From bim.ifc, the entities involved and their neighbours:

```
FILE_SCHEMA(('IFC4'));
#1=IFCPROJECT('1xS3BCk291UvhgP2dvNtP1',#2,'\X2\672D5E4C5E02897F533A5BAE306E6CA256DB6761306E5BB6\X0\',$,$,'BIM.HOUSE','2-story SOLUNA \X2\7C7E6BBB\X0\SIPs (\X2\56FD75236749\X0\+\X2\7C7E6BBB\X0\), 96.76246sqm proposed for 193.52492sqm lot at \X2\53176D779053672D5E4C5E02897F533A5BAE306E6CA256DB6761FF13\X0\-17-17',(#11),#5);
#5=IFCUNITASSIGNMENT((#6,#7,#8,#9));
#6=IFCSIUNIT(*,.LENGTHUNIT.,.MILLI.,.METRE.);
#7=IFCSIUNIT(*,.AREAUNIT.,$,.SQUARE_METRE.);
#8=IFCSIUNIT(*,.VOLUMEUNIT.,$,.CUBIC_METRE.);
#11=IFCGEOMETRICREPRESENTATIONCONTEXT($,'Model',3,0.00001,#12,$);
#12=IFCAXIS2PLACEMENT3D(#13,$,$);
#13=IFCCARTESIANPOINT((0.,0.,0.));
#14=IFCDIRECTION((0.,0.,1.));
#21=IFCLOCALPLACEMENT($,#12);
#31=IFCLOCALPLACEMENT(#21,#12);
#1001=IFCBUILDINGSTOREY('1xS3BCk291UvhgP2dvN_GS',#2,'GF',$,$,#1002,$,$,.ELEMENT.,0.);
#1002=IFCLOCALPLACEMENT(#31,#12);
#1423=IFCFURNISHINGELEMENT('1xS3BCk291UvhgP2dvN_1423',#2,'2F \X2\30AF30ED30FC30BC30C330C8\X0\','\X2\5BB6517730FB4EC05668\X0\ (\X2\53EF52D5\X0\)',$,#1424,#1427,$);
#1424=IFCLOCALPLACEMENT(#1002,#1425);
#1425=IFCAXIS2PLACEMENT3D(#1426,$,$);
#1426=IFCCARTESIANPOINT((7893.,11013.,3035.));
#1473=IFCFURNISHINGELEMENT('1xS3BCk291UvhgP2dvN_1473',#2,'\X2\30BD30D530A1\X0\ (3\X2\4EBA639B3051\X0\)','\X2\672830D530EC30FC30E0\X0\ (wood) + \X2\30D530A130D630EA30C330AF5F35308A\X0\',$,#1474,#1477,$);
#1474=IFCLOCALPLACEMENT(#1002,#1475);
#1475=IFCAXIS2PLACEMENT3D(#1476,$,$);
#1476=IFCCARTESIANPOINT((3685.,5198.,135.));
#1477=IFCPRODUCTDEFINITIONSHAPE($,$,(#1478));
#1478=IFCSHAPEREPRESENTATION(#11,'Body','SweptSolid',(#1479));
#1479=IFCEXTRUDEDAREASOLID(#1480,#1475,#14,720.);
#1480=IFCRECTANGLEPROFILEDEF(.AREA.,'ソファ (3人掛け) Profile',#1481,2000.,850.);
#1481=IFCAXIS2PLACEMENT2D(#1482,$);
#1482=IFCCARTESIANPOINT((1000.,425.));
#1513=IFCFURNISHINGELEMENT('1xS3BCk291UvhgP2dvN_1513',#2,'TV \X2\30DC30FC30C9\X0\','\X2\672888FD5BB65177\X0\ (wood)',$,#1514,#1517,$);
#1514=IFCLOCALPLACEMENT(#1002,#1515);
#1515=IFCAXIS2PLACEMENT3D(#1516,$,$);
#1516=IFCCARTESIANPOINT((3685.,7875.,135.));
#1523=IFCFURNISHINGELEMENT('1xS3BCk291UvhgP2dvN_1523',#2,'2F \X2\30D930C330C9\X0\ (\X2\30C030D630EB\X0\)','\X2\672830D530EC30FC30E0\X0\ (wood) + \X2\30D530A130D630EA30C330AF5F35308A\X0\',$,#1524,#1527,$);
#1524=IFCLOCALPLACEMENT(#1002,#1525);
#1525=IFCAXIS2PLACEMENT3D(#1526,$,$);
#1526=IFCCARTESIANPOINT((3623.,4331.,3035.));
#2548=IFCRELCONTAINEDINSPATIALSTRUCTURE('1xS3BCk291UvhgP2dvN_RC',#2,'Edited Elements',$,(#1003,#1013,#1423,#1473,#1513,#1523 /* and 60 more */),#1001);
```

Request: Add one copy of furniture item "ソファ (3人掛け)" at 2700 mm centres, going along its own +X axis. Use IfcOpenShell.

```python
import ifcopenshell
import ifcopenshell.api.geometry
import ifcopenshell.api.root
import ifcopenshell.util.element
import ifcopenshell.util.placement
import ifcopenshell.util.unit

model = ifcopenshell.open("bim.ifc")
unit_scale = ifcopenshell.util.unit.calculate_unit_scale(model)


def reuse_history(source, copy):
    """copy_class also copies each property set's owner history, people and application; keep the originals."""
    for rel in copy.IsDefinedBy:
        if rel.is_a("IfcRelDefinesByProperties") and (history := rel.RelatingPropertyDefinition.OwnerHistory):
            rel.RelatingPropertyDefinition.OwnerHistory = source.OwnerHistory
            ifcopenshell.util.element.remove_deep2(model, history)


source = model.by_guid("1xS3BCk291UvhgP2dvN_1473")
base = ifcopenshell.util.placement.get_local_placement(source.ObjectPlacement)
step = base[:3, 0] * 2.7 / unit_scale

for i in range(1, 2):
    copy = ifcopenshell.api.root.copy_class(model, product=source)
    copy.Representation = ifcopenshell.util.element.copy_deep(
        model, source.Representation, exclude=["IfcGeometricRepresentationContext", "IfcRepresentationMap"]
    )
    reuse_history(source, copy)
    matrix = base.copy()
    matrix[:3, 3] += i * step
    print("added at", matrix[:3, 3].round(3) + 0.0)
    ifcopenshell.api.geometry.edit_object_placement(model, product=copy, matrix=matrix, is_si=False)

model.write("bim-out.ifc")
```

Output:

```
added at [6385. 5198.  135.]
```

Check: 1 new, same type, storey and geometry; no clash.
